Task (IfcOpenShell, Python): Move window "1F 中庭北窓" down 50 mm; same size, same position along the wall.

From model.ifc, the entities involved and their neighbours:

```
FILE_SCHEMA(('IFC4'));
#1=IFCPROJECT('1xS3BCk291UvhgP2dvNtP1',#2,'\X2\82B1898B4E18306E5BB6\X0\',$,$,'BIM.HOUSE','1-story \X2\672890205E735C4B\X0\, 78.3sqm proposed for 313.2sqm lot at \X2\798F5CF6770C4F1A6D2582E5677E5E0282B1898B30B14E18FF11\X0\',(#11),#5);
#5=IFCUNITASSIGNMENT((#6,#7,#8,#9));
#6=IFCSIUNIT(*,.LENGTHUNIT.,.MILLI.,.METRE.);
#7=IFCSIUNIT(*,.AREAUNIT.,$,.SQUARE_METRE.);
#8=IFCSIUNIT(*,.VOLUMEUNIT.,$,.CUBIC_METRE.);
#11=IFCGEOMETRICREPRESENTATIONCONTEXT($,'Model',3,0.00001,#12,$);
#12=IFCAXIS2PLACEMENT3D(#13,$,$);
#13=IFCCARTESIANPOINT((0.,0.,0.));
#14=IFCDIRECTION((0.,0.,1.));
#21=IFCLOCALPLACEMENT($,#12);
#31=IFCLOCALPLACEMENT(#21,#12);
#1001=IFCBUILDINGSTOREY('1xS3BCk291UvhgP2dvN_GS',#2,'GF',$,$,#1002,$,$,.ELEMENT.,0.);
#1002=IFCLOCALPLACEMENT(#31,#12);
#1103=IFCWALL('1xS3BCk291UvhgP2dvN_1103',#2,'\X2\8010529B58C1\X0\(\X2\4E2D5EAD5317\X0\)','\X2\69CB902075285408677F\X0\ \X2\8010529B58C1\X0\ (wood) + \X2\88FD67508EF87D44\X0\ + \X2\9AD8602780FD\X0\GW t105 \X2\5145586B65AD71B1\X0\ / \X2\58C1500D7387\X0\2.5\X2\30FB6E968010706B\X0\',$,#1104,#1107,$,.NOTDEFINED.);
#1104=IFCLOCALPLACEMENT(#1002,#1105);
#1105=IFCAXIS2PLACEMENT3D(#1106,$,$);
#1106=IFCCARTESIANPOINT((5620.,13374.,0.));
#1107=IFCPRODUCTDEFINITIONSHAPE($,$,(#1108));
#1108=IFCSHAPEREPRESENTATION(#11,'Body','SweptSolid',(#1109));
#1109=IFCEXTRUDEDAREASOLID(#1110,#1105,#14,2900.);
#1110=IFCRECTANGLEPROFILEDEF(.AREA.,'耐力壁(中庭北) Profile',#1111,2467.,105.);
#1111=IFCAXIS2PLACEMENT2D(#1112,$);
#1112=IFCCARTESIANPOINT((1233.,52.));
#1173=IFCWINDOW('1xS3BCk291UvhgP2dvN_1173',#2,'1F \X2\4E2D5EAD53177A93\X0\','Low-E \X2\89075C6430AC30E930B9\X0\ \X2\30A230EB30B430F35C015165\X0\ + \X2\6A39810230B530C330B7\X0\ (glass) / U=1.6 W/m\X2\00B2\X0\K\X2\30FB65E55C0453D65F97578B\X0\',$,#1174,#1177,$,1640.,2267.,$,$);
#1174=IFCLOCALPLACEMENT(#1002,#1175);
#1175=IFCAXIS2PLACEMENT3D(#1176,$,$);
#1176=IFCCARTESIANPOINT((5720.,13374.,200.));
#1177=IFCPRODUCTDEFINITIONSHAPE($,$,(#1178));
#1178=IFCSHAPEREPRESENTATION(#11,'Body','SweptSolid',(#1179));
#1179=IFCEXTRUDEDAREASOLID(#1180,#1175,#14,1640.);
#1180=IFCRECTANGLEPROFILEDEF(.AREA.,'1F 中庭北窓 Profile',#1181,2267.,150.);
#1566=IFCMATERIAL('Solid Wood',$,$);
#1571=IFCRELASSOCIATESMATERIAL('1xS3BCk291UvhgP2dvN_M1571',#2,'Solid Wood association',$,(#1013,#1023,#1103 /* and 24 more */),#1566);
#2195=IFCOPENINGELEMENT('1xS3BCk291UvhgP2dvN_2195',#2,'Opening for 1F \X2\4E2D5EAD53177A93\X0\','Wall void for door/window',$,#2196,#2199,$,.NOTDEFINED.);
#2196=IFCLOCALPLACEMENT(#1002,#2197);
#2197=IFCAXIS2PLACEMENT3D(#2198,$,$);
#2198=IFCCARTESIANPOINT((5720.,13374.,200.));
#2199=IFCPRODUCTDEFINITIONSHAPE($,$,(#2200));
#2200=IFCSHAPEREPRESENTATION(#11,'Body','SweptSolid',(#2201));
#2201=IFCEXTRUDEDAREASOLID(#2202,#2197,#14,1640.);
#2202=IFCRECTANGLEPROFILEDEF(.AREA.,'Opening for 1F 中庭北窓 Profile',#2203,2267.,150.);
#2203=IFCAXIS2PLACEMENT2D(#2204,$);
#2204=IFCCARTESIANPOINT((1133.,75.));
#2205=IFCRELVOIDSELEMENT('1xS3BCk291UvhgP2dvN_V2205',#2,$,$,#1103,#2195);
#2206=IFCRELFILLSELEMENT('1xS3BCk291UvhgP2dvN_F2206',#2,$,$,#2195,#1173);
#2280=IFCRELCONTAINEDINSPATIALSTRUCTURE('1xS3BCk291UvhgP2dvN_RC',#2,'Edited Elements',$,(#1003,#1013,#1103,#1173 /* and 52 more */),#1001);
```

```python
import numpy as np
import ifcopenshell
import ifcopenshell.api.geometry
import ifcopenshell.util.placement
import ifcopenshell.util.unit

model = ifcopenshell.open("model.ifc")
unit_scale = ifcopenshell.util.unit.calculate_unit_scale(model)

window = model.by_guid("1xS3BCk291UvhgP2dvN_1173")
opening = window.FillsVoids[0].RelatingOpeningElement
dz = -0.05 / unit_scale

shift = np.array([0.0, 0.0, dz])
# The window is not placed relative to its opening, so move both.
for product in (opening, window):
    matrix = ifcopenshell.util.placement.get_local_placement(product.ObjectPlacement)
    matrix[:3, 3] += shift
    ifcopenshell.api.geometry.edit_object_placement(model, product=product, matrix=matrix, is_si=False)

print(f"moved by {dz * unit_scale:+.3f} m")

model.write("model_edited.ifc")
```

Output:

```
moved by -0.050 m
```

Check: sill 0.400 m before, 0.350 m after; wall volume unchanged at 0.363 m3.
